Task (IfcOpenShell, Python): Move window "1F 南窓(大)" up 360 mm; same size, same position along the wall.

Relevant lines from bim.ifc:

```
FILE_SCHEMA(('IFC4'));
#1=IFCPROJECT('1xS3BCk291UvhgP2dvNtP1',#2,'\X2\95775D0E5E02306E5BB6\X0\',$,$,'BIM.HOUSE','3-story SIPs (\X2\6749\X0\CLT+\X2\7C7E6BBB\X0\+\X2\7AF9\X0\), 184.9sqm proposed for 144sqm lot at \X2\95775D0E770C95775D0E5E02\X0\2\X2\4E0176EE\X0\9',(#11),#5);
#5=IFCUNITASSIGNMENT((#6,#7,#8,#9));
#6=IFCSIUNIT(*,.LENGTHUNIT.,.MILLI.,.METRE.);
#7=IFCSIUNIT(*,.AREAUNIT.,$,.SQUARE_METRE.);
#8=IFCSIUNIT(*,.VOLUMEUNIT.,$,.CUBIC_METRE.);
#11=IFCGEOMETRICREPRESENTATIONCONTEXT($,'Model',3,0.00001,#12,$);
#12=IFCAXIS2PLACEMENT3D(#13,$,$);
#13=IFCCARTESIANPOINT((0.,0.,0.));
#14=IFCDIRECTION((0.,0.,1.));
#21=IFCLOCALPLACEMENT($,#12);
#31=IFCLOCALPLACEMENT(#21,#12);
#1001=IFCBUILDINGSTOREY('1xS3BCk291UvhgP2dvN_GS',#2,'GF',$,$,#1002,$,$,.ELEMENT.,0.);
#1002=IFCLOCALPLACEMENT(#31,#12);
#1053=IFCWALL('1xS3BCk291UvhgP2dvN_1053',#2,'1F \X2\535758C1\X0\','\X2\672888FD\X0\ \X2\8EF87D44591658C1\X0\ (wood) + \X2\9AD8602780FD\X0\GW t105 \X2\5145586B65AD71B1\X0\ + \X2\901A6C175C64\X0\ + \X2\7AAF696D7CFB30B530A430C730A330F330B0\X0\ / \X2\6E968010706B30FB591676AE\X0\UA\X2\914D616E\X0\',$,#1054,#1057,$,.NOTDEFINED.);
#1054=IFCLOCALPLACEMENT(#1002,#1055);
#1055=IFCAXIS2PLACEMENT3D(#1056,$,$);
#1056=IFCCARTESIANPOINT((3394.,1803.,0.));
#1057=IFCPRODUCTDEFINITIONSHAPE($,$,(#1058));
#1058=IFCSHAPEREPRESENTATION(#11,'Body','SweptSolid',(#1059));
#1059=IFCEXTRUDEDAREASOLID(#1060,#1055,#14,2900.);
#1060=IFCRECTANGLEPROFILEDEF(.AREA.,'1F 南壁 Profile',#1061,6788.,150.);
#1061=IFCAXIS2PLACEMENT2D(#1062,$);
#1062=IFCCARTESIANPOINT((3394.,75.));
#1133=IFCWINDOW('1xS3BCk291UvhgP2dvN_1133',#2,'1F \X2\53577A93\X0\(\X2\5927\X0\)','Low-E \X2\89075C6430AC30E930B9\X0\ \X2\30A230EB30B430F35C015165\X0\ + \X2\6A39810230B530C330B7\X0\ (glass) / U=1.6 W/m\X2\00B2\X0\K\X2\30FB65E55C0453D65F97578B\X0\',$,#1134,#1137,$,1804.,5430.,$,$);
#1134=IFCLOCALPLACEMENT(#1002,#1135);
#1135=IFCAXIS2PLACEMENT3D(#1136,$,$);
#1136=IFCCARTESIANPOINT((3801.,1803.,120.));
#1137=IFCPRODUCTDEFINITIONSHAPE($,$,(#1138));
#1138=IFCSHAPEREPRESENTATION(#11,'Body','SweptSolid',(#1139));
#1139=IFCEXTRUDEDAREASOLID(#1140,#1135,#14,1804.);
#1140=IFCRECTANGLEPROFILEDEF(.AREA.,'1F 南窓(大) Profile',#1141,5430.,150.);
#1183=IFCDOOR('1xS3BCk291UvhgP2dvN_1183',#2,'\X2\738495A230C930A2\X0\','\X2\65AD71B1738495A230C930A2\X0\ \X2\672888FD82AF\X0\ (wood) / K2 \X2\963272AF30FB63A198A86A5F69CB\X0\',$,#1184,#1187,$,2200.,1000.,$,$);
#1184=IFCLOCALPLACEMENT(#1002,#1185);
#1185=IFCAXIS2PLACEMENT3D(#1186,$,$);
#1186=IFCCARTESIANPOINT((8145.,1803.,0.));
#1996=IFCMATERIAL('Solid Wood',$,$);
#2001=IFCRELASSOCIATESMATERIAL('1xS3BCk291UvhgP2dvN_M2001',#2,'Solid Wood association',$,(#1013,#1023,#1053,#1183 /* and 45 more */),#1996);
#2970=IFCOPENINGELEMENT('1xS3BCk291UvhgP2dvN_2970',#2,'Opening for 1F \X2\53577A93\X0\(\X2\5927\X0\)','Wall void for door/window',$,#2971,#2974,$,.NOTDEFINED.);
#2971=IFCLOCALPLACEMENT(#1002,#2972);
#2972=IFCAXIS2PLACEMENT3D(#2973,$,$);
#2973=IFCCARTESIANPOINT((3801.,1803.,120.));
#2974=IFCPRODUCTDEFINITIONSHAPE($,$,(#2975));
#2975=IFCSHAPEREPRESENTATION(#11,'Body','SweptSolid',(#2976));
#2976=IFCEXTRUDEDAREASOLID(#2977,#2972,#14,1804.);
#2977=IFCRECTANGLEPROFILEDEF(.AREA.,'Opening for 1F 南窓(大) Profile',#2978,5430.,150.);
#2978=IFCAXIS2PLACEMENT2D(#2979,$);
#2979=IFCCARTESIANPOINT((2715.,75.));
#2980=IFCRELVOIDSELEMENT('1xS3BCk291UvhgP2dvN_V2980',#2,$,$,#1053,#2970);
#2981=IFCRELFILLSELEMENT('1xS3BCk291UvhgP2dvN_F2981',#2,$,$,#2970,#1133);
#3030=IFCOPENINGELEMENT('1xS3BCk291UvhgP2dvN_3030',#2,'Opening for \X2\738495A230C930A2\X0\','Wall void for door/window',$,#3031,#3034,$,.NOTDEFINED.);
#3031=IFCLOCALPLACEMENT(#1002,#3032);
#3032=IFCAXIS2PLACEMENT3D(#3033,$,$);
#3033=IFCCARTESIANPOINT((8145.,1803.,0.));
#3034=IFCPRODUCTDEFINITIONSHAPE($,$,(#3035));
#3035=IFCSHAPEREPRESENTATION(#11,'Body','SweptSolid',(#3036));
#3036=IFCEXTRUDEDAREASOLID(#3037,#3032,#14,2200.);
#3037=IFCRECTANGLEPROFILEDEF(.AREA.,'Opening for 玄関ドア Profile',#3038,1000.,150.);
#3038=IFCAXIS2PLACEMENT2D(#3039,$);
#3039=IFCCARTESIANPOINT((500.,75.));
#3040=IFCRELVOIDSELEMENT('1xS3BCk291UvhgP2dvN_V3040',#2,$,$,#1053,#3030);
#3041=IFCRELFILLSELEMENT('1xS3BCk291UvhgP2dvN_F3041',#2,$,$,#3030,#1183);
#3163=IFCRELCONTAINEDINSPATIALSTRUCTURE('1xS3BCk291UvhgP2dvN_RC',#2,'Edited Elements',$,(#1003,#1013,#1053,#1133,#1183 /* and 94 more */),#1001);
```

```python
import numpy as np
import ifcopenshell
import ifcopenshell.api.geometry
import ifcopenshell.util.placement
import ifcopenshell.util.unit

model = ifcopenshell.open("bim.ifc")
unit_scale = ifcopenshell.util.unit.calculate_unit_scale(model)

window = model.by_guid("1xS3BCk291UvhgP2dvN_1133")
opening = window.FillsVoids[0].RelatingOpeningElement
dz = 0.36 / unit_scale

shift = np.array([0.0, 0.0, dz])
# The window is not placed relative to its opening, so move both.
for product in (opening, window):
    matrix = ifcopenshell.util.placement.get_local_placement(product.ObjectPlacement)
    matrix[:3, 3] += shift
    ifcopenshell.api.geometry.edit_object_placement(model, product=product, matrix=matrix, is_si=False)

print(f"moved by {dz * unit_scale:+.3f} m")

model.write("bim-out.ifc")
```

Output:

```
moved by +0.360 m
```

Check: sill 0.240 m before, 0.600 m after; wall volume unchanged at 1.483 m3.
